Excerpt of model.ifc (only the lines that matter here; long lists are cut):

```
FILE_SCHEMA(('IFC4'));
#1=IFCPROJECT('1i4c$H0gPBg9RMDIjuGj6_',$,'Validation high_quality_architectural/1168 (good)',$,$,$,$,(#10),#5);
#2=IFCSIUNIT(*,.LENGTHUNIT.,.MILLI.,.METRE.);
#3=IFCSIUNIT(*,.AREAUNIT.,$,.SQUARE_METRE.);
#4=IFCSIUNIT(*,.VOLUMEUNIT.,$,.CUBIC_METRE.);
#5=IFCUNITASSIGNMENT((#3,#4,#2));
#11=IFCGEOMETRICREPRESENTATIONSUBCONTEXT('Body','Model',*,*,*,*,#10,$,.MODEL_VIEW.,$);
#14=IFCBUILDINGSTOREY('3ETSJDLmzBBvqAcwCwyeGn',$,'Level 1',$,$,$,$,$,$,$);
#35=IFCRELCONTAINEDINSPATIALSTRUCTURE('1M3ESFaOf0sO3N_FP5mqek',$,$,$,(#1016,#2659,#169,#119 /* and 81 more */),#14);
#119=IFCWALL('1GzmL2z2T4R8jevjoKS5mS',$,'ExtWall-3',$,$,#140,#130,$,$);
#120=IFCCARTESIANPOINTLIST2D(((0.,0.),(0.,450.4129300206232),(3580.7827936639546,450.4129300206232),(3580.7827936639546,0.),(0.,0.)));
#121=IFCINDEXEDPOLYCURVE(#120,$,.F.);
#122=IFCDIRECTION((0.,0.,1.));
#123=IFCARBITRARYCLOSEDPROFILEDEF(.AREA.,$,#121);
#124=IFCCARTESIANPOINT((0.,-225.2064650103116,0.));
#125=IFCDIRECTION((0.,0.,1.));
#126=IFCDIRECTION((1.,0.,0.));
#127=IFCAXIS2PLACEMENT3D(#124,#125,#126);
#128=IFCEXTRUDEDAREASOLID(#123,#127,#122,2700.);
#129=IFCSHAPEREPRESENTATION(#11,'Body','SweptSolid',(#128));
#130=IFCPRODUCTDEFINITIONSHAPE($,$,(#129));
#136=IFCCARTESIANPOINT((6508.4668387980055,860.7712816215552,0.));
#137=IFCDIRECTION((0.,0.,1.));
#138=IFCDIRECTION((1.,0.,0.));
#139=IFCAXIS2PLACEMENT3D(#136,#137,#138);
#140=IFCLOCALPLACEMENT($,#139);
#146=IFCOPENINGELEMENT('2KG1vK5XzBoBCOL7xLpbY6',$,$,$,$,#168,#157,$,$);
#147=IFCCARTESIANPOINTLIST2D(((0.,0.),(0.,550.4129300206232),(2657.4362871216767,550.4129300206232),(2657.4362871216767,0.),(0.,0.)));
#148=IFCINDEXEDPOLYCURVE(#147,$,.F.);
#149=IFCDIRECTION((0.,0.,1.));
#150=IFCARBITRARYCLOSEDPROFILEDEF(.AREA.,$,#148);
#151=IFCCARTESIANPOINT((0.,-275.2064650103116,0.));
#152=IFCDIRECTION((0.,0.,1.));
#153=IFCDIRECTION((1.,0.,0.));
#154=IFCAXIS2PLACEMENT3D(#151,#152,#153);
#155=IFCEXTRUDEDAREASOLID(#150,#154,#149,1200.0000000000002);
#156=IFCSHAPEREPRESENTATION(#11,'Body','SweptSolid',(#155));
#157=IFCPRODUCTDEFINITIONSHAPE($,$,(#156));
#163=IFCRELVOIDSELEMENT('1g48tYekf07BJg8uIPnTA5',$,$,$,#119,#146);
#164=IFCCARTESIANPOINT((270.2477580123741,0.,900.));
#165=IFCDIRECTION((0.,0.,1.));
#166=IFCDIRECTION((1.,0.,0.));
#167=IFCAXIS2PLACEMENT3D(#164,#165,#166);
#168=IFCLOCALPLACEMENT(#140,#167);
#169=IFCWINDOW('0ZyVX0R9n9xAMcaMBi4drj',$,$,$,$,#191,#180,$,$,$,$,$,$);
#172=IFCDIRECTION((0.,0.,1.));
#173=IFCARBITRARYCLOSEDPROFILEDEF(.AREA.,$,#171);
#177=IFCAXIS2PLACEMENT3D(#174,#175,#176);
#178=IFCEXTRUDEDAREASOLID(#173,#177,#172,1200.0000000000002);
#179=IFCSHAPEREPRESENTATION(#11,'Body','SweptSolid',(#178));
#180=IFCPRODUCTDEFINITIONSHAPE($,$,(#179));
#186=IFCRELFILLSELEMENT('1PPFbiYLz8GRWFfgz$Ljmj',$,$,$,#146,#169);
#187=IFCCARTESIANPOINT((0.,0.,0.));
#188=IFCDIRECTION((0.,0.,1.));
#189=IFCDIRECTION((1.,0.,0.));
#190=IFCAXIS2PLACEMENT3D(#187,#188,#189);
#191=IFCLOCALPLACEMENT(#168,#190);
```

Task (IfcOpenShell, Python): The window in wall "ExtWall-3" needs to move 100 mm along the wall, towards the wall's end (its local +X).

```python
import ifcopenshell
import ifcopenshell.api.geometry
import ifcopenshell.util.placement

model = ifcopenshell.open("model.ifc")

window = model.by_guid("0ZyVX0R9n9xAMcaMBi4drj")
opening = window.FillsVoids[0].RelatingOpeningElement
wall = opening.VoidsElements[0].RelatingBuildingElement

wall_matrix = ifcopenshell.util.placement.get_local_placement(wall.ObjectPlacement)
shift = wall_matrix[:3, 0] * 100.0
before = ifcopenshell.util.placement.get_local_placement(window.ObjectPlacement)[:3, 3].copy()

# The window is placed relative to its opening, so it follows when the opening moves.
matrix = ifcopenshell.util.placement.get_local_placement(opening.ObjectPlacement)
matrix[:3, 3] += shift
ifcopenshell.api.geometry.edit_object_placement(
    model, product=opening, matrix=matrix, is_si=False, should_transform_children=True
)

after = ifcopenshell.util.placement.get_local_placement(window.ObjectPlacement)[:3, 3]
print("window moved by", (after - before).round(3) + 0.0)

model.write("model_v2.ifc")
```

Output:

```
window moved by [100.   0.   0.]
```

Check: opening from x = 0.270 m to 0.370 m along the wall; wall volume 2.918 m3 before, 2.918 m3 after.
